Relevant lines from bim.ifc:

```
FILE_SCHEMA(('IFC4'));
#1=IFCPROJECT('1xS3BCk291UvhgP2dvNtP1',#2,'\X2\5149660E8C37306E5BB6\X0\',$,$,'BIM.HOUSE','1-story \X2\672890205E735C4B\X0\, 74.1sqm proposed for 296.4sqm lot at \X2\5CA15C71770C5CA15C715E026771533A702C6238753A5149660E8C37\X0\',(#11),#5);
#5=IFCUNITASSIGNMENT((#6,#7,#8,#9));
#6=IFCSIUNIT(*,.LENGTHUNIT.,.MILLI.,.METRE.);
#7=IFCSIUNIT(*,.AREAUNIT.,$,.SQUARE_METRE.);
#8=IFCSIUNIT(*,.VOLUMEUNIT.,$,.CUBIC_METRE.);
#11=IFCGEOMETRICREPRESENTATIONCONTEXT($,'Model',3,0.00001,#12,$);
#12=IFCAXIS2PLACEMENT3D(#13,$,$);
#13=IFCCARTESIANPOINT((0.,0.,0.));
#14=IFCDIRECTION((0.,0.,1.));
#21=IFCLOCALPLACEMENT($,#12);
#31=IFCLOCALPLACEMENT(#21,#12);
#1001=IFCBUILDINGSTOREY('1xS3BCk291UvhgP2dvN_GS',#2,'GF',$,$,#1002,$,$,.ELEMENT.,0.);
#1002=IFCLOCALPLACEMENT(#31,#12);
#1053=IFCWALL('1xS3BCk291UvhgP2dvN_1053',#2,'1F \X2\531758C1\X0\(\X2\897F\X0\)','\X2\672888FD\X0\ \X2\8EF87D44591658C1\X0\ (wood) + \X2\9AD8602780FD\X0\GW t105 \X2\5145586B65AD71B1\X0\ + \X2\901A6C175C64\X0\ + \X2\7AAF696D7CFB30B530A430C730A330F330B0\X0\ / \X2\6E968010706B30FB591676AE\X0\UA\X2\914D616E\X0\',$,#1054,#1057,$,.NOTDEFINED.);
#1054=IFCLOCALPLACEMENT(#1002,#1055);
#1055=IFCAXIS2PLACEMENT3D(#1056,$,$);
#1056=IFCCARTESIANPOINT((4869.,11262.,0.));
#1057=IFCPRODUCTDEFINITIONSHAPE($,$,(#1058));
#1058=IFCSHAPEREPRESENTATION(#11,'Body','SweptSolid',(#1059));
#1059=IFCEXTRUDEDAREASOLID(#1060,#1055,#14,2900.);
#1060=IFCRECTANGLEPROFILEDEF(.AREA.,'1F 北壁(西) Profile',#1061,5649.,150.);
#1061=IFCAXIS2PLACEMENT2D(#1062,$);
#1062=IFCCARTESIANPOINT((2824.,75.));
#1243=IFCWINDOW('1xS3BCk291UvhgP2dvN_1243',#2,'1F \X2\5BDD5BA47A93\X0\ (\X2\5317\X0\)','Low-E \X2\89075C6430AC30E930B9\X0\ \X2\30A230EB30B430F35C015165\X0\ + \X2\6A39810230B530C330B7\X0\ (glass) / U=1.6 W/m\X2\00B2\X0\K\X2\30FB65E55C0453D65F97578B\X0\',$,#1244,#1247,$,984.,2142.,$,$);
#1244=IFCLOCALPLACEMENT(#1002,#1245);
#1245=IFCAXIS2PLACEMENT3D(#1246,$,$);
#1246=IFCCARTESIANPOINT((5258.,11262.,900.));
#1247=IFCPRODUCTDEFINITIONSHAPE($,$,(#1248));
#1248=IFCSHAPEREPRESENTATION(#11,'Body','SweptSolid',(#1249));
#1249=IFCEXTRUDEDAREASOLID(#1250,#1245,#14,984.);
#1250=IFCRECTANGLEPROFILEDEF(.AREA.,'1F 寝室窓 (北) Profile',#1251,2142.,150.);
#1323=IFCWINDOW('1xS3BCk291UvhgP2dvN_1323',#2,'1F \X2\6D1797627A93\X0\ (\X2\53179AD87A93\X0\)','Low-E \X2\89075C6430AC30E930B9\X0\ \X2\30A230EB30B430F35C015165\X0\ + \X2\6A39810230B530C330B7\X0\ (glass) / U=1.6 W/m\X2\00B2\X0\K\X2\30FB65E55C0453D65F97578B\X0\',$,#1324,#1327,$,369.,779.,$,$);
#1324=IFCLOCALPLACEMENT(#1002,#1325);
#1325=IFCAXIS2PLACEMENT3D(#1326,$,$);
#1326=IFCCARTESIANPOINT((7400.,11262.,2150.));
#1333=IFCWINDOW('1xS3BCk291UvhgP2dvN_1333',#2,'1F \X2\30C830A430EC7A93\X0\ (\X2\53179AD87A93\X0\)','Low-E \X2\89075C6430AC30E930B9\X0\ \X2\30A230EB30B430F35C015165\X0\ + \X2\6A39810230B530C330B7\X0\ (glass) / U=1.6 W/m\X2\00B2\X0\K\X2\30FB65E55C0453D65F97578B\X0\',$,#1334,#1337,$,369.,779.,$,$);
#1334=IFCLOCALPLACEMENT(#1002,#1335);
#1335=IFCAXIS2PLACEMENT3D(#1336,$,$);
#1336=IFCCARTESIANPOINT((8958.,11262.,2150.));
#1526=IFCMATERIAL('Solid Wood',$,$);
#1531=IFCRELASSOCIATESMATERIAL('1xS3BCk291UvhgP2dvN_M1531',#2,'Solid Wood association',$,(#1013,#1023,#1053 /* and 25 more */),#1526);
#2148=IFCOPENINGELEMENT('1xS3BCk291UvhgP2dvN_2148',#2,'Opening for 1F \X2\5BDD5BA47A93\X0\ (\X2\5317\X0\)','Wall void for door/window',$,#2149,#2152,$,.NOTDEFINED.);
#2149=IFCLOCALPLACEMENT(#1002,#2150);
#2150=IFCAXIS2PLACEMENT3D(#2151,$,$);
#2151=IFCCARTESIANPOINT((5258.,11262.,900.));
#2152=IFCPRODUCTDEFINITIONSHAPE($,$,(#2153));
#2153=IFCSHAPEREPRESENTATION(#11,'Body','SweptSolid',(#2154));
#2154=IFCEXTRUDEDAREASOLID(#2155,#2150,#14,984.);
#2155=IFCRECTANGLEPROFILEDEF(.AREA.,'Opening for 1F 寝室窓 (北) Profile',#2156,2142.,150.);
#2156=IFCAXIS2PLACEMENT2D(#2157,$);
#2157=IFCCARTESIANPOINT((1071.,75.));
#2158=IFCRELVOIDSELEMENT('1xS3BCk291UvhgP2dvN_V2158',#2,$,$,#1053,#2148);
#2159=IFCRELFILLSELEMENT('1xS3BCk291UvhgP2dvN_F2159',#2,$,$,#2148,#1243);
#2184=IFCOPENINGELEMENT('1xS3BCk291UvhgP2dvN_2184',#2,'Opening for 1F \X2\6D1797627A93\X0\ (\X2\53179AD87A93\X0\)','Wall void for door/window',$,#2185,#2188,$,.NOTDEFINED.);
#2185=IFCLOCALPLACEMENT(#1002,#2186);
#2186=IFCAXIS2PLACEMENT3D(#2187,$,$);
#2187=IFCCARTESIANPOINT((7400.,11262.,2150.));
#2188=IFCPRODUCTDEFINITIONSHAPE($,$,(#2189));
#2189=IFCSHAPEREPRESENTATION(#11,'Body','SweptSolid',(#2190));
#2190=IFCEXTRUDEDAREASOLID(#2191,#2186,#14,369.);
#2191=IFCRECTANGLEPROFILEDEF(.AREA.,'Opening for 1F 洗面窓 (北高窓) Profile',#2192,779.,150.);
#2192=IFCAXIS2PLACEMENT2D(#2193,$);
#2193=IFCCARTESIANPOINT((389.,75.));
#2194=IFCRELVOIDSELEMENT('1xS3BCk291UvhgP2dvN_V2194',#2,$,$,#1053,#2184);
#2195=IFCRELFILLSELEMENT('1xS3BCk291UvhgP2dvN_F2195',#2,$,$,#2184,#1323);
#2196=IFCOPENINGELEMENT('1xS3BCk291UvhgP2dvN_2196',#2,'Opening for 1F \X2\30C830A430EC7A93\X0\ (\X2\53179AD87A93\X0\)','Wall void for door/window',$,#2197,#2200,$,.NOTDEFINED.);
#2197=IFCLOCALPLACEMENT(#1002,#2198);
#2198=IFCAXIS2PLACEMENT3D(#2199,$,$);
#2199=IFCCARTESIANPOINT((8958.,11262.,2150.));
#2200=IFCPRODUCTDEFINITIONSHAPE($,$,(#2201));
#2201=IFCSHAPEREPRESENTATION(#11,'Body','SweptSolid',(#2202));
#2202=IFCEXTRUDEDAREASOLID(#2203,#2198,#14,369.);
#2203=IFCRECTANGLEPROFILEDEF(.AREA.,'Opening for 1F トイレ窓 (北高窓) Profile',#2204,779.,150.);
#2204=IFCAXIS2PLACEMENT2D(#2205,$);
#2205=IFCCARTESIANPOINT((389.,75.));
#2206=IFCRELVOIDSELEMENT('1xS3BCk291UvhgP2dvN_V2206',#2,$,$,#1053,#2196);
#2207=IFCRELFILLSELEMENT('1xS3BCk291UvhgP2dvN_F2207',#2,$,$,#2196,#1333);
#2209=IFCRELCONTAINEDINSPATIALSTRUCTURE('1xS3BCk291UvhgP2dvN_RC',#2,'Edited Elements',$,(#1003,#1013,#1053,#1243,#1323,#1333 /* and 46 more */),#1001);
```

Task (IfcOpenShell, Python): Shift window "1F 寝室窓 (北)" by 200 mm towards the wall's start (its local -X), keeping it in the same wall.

```python
import ifcopenshell
import ifcopenshell.api.geometry
import ifcopenshell.util.placement
import ifcopenshell.util.unit

model = ifcopenshell.open("bim.ifc")
unit_scale = ifcopenshell.util.unit.calculate_unit_scale(model)

window = model.by_guid("1xS3BCk291UvhgP2dvN_1243")
opening = window.FillsVoids[0].RelatingOpeningElement
wall = opening.VoidsElements[0].RelatingBuildingElement

wall_matrix = ifcopenshell.util.placement.get_local_placement(wall.ObjectPlacement)
shift = wall_matrix[:3, 0] * -0.2 / unit_scale
before = ifcopenshell.util.placement.get_local_placement(window.ObjectPlacement)[:3, 3].copy()

# The window is not placed relative to its opening, so move both.
for product in (opening, window):
    matrix = ifcopenshell.util.placement.get_local_placement(product.ObjectPlacement)
    matrix[:3, 3] += shift
    ifcopenshell.api.geometry.edit_object_placement(model, product=product, matrix=matrix, is_si=False)

after = ifcopenshell.util.placement.get_local_placement(window.ObjectPlacement)[:3, 3]
print("window moved by", (after - before).round(3) + 0.0)

model.write("bim_rev.ifc")
```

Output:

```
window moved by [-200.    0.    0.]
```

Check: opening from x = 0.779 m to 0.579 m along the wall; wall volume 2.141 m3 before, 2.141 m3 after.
